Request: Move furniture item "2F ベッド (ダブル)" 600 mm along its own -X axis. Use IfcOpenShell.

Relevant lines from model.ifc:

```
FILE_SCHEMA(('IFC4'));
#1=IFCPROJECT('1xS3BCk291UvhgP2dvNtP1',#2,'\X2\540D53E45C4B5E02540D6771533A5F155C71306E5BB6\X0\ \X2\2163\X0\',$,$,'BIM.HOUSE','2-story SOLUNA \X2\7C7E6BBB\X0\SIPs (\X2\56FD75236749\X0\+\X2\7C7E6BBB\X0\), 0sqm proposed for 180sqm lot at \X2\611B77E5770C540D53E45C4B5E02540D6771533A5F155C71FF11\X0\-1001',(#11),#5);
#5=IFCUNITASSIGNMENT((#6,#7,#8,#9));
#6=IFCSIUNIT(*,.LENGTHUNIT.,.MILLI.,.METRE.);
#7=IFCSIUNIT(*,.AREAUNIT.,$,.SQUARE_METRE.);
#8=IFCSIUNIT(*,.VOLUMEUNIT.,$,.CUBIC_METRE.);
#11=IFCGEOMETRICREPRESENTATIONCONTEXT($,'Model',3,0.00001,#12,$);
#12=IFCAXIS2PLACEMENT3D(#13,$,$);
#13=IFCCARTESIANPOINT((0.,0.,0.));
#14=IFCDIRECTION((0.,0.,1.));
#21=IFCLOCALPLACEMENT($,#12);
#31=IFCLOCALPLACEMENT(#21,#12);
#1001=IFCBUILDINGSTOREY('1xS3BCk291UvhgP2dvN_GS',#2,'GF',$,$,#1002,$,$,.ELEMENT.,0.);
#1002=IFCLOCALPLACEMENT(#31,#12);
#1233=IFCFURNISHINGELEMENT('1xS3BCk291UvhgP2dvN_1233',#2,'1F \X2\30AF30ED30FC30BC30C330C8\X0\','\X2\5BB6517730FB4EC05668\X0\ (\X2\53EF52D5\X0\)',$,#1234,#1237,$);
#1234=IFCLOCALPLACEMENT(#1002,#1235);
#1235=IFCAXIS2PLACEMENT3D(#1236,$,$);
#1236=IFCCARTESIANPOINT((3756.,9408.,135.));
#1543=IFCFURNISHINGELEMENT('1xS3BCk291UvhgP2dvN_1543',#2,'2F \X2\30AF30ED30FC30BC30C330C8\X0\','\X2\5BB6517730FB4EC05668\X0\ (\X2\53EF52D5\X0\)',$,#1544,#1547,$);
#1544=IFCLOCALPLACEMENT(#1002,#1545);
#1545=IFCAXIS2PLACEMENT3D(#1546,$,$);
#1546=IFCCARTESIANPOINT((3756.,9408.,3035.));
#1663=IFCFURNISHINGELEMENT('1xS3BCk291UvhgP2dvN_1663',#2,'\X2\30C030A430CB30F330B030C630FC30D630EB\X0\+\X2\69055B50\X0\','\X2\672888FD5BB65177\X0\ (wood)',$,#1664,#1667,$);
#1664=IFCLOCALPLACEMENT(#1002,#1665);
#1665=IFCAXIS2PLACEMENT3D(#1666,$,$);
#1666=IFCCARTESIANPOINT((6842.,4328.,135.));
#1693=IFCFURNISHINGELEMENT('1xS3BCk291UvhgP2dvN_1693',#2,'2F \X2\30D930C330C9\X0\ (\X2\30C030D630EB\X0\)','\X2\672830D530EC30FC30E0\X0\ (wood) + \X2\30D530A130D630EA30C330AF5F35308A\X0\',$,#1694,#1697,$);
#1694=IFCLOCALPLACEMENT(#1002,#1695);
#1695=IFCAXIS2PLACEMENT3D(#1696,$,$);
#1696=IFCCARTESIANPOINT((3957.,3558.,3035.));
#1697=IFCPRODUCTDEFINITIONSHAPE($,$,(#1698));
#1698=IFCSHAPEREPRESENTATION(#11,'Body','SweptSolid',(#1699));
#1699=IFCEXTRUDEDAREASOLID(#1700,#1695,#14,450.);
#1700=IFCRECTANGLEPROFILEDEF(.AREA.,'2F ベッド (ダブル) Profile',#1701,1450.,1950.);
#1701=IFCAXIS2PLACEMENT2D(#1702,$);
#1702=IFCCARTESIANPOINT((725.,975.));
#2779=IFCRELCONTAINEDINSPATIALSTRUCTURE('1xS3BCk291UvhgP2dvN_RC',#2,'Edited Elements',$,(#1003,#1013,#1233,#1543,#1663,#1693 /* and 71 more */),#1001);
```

```python
import ifcopenshell
import ifcopenshell.api.geometry
import ifcopenshell.util.placement
import ifcopenshell.util.unit

model = ifcopenshell.open("model.ifc")
unit_scale = ifcopenshell.util.unit.calculate_unit_scale(model)

item = model.by_guid("1xS3BCk291UvhgP2dvN_1693")
matrix = ifcopenshell.util.placement.get_local_placement(item.ObjectPlacement)
matrix[:3, 3] -= matrix[:3, 0] * 0.6 / unit_scale
ifcopenshell.api.geometry.edit_object_placement(model, product=item, matrix=matrix, is_si=False)

print(ifcopenshell.util.placement.get_local_placement(item.ObjectPlacement).round(3) + 0.0)

model.write("model_rev.ifc")
```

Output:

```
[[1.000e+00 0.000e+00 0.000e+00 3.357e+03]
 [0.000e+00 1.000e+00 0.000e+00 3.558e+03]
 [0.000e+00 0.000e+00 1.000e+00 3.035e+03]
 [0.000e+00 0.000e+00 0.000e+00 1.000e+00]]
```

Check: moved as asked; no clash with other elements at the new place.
